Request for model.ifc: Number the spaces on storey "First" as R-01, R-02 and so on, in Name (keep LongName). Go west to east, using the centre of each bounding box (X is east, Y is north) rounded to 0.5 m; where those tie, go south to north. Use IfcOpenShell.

First a look at what the model holds.

```python
import ifcopenshell
import ifcopenshell.util.element
import ifcopenshell.util.placement

model = ifcopenshell.open("model.ifc")
print(model.schema)
storey = next(s for s in model.by_type("IfcBuildingStorey") if s.Name == "First")
spaces = [e for e in ifcopenshell.util.element.get_decomposition(storey) if e.is_a("IfcSpace")]
for e in sorted(spaces, key=lambda e: e.id()):
    origin = ifcopenshell.util.placement.get_local_placement(e.ObjectPlacement)[:3, 3]
    print(e.id(), e.Name, e.LongName, origin.round(2) + 0.0, sep=" | ")
```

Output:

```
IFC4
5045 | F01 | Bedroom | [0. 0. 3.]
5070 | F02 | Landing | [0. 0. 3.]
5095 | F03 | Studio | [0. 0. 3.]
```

```python
import ifcopenshell
import ifcopenshell.geom
import ifcopenshell.util.element
import ifcopenshell.util.shape

model = ifcopenshell.open("model.ifc")
settings = ifcopenshell.geom.settings()
settings.set("use-world-coords", True)


def centre(element):
    shape = ifcopenshell.geom.create_shape(settings, element)
    return ifcopenshell.util.shape.get_bbox_centroid(shape.geometry)


storey = next(s for s in model.by_type("IfcBuildingStorey") if s.Name == "First")
spaces = [e for e in ifcopenshell.util.element.get_decomposition(storey) if e.is_a("IfcSpace")]

# Insertion points can sit at a corner or the storey origin, so sort by the geometry (in metres).
centres = {e: centre(e) for e in spaces}
spaces.sort(key=lambda e: (round(centres[e][0] / 0.5), centres[e][1]))

for i, e in enumerate(spaces, start=1):
    number = f"R-{i:02d}"
    e.Name = number
    print(e.id(), number)

model.write("model_edited.ifc")
```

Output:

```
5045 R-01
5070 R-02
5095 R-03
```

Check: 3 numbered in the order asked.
